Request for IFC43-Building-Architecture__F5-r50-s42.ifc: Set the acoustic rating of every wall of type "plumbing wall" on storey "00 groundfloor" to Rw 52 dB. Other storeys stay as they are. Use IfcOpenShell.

First a look at what the model holds.

```python
import ifcopenshell
import ifcopenshell.util.element

model = ifcopenshell.open("IFC43-Building-Architecture__F5-r50-s42.ifc")
print(model.schema)
storey = next(s for s in model.by_type("IfcBuildingStorey") if s.Name == "00 groundfloor")
walls = [e for e in ifcopenshell.util.element.get_decomposition(storey) if e.is_a("IfcWall")]
seen = {}
for e in walls:
    element_type = ifcopenshell.util.element.get_type(e)
    key = (element_type.Name if element_type != e and element_type else None, ifcopenshell.util.element.get_pset(e, "Pset_WallCommon", "AcousticRating"))
    seen[key] = seen.get(key, 0) + 1
for (name, value), count in sorted(seen.items(), key=str):
    print(count, "x", name, "|", value)
```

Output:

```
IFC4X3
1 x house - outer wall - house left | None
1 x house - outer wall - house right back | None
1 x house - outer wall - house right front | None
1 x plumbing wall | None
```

```python
import ifcopenshell
import ifcopenshell.api.pset
import ifcopenshell.util.element

model = ifcopenshell.open("IFC43-Building-Architecture__F5-r50-s42.ifc")

storey = next(s for s in model.by_type("IfcBuildingStorey") if s.Name == "00 groundfloor")
walls = [e for e in ifcopenshell.util.element.get_decomposition(storey) if e.is_a("IfcWall")]

count = 0
for e in walls:
    element_type = ifcopenshell.util.element.get_type(e)
    if element_type in (None, e) or element_type.Name != "plumbing wall":
        continue
    # add_pset returns the element's existing set when there is one.
    pset = ifcopenshell.api.pset.add_pset(model, product=e, name="Pset_WallCommon")
    ifcopenshell.api.pset.edit_pset(model, pset=pset, properties={"AcousticRating": "Rw 52 dB"})
    count += 1

print(count, "walls updated")

model.write("IFC43-Building-Architecture__F5-r50-s42-out.ifc")
```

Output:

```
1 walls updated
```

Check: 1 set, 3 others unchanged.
